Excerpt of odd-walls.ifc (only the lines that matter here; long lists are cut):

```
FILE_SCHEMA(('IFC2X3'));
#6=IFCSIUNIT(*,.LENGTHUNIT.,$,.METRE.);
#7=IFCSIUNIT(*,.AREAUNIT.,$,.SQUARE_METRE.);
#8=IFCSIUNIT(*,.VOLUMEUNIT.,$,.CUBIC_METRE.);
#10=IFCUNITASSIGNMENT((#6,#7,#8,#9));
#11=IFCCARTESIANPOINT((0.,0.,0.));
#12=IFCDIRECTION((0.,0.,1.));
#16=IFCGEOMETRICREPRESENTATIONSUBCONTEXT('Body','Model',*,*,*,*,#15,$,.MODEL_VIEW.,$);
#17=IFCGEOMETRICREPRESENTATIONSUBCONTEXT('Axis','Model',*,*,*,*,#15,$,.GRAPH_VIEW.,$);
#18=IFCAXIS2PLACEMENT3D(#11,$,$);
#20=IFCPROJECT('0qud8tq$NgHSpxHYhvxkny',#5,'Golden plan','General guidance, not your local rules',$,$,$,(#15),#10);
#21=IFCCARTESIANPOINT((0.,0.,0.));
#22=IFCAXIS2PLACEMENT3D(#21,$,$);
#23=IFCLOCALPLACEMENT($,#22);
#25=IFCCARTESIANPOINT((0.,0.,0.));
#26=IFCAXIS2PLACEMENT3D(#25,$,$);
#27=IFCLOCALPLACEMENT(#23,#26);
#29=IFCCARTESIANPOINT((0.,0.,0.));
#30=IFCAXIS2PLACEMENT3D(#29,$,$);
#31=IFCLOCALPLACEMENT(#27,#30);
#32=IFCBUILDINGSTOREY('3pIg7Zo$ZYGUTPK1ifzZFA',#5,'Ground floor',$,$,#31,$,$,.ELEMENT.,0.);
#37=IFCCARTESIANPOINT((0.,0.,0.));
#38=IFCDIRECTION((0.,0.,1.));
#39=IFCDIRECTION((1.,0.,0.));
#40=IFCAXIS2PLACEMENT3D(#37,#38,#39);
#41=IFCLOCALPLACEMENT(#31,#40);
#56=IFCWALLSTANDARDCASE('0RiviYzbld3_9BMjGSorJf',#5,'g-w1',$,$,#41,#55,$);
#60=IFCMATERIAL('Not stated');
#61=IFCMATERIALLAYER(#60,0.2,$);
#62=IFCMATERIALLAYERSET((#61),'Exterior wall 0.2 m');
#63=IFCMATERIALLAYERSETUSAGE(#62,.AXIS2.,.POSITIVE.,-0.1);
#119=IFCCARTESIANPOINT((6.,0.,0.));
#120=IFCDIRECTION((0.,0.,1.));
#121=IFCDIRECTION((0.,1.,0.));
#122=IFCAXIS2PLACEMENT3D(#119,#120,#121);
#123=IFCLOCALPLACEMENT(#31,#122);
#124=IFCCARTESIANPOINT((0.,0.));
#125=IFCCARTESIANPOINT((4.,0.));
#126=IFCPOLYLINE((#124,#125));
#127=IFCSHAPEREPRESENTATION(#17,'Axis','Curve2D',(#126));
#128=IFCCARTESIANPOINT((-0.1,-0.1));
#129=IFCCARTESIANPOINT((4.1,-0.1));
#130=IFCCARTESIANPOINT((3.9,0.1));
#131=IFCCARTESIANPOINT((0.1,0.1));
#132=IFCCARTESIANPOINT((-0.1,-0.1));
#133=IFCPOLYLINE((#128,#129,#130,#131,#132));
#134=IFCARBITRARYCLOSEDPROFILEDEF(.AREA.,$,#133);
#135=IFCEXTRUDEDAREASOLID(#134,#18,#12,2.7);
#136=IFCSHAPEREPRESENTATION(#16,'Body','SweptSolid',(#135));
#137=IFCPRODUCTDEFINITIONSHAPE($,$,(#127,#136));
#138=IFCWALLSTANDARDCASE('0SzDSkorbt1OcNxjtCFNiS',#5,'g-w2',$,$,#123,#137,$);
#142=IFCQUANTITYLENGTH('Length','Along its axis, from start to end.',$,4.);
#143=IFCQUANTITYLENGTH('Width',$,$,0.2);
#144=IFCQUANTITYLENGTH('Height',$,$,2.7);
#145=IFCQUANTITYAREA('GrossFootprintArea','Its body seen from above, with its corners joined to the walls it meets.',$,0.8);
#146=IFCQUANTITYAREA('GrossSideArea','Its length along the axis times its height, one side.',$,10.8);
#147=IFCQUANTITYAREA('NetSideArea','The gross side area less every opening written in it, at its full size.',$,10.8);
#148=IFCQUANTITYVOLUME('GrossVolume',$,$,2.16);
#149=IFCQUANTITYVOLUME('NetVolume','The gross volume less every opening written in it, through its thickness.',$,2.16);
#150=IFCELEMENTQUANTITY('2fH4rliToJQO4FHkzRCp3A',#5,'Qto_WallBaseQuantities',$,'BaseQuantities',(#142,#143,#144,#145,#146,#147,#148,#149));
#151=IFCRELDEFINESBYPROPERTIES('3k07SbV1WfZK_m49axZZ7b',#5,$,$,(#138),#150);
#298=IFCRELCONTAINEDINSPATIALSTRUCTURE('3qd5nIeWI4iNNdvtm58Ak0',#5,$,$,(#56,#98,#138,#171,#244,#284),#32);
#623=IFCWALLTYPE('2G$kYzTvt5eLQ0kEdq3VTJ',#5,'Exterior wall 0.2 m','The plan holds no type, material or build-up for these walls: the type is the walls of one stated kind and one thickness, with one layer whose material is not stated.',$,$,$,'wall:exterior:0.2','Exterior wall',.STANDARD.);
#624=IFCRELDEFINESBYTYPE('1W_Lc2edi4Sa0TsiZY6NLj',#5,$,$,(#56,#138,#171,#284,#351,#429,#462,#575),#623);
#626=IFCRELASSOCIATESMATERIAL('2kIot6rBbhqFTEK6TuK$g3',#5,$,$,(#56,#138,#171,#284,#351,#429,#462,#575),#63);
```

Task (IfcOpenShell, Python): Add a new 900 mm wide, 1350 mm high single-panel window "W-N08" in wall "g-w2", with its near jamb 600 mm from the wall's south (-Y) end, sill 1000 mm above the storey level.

```python
import numpy as np
import ifcopenshell
import ifcopenshell.api.feature
import ifcopenshell.api.geometry
import ifcopenshell.api.pset
import ifcopenshell.api.root
import ifcopenshell.api.spatial
import ifcopenshell.api.type
import ifcopenshell.geom
import ifcopenshell.util.element
import ifcopenshell.util.placement
import ifcopenshell.util.representation
import ifcopenshell.util.shape
import ifcopenshell.util.unit

model = ifcopenshell.open("odd-walls.ifc")
unit_scale = ifcopenshell.util.unit.calculate_unit_scale(model)
area_scale = ifcopenshell.util.unit.calculate_unit_scale(model, "AREAUNIT")
volume_scale = ifcopenshell.util.unit.calculate_unit_scale(model, "VOLUMEUNIT")
settings = ifcopenshell.geom.settings()


def volume(element):
    """Net volume in cubic metres, openings subtracted."""
    shape = ifcopenshell.geom.create_shape(settings, element)
    return ifcopenshell.util.shape.get_volume(shape.geometry)


wall = model.by_guid("0SzDSkorbt1OcNxjtCFNiS")
storey = ifcopenshell.util.element.get_container(wall, ifc_class="IfcBuildingStorey")
context = ifcopenshell.util.representation.get_context(model, "Model", "Body", "MODEL_VIEW")
before = volume(wall)

width, height, from_end, sill = 0.9, 1.35, 0.6, 1  # metres

# The wall runs along its own X axis, and the end named is its -X end.
wall_shape = ifcopenshell.geom.create_shape(settings, wall)
x, y, z = ifcopenshell.util.shape.get_vertices(wall_shape.geometry).T
start = x.min() + from_end
face, thickness = float(y.min()), float(y.max() - y.min())
wall_matrix = ifcopenshell.util.placement.get_local_placement(wall.ObjectPlacement)
level = ifcopenshell.util.placement.get_local_placement(storey.ObjectPlacement)[2, 3]


def in_wall(x, y):
    """Placement at x, y metres in the wall's axes, at sill height."""
    matrix = wall_matrix.copy()
    matrix[:, 3] = wall_matrix @ np.array([x / unit_scale, y / unit_scale, 0.0, 1.0])
    matrix[2, 3] = level + sill / unit_scale
    return matrix


# Opening: a box that overshoots both wall faces by 50 mm.
opening = ifcopenshell.api.root.create_entity(model, ifc_class="IfcOpeningElement")
box = ifcopenshell.api.geometry.add_wall_representation(
    model, context=context, length=width, height=height, thickness=thickness + 0.1
)
ifcopenshell.api.geometry.assign_representation(model, product=opening, representation=box)
ifcopenshell.api.geometry.edit_object_placement(model, product=opening, matrix=in_wall(start, face - 0.05), is_si=False)
ifcopenshell.api.feature.add_feature(model, feature=opening, element=wall)

window = ifcopenshell.api.root.create_entity(model, ifc_class="IfcWindow", name="W-N08")
window.OverallWidth, window.OverallHeight = width / unit_scale, height / unit_scale
body = ifcopenshell.api.geometry.add_window_representation(
    model,
    context=context,
    overall_width=window.OverallWidth,
    overall_height=window.OverallHeight,
    partition_type="SINGLE_PANEL",
)
ifcopenshell.api.geometry.assign_representation(model, product=window, representation=body)
ifcopenshell.api.spatial.assign_container(model, products=[window], relating_structure=storey)
fills = ifcopenshell.api.feature.add_filling(model, opening=opening, element=window)
fills.OwnerHistory = window.OwnerHistory  # required in IFC2X3

# IFC2X3 keeps the operation on the window style.
style = ifcopenshell.api.root.create_entity(model, ifc_class="IfcWindowStyle", name="W-N08")
style.OperationType, style.ConstructionType = "SINGLE_PANEL", "NOTDEFINED"
style.ParameterTakesPrecedence = style.Sizeable = False
ifcopenshell.api.type.assign_type(model, related_objects=[window], relating_type=style)

# Centre the window in the wall's thickness.
ifcopenshell.api.geometry.edit_object_placement(model, product=window, matrix=in_wall(start, face), is_si=False)
window_shape = ifcopenshell.geom.create_shape(settings, window)
depth = ifcopenshell.util.shape.get_vertices(window_shape.geometry)[:, 1]
offset = face + thickness / 2 - (depth.min() + depth.max()) / 2
ifcopenshell.api.geometry.edit_object_placement(model, product=window, matrix=in_wall(start, offset), is_si=False)

after = volume(wall)

# Update the wall's stored quantities.
qto = model.by_id(ifcopenshell.util.element.get_pset(wall, "Qto_WallBaseQuantities", should_inherit=False)["id"])
ifcopenshell.api.pset.edit_qto(model, qto=qto, properties={
    "NetSideArea": after / thickness / area_scale,
    "NetVolume": after / volume_scale,
})

print(f"wall volume {before:.3f} -> {after:.3f} m3")

model.write("odd-walls-out.ifc")
```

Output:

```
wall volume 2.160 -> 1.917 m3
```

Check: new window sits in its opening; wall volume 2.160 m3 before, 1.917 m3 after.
